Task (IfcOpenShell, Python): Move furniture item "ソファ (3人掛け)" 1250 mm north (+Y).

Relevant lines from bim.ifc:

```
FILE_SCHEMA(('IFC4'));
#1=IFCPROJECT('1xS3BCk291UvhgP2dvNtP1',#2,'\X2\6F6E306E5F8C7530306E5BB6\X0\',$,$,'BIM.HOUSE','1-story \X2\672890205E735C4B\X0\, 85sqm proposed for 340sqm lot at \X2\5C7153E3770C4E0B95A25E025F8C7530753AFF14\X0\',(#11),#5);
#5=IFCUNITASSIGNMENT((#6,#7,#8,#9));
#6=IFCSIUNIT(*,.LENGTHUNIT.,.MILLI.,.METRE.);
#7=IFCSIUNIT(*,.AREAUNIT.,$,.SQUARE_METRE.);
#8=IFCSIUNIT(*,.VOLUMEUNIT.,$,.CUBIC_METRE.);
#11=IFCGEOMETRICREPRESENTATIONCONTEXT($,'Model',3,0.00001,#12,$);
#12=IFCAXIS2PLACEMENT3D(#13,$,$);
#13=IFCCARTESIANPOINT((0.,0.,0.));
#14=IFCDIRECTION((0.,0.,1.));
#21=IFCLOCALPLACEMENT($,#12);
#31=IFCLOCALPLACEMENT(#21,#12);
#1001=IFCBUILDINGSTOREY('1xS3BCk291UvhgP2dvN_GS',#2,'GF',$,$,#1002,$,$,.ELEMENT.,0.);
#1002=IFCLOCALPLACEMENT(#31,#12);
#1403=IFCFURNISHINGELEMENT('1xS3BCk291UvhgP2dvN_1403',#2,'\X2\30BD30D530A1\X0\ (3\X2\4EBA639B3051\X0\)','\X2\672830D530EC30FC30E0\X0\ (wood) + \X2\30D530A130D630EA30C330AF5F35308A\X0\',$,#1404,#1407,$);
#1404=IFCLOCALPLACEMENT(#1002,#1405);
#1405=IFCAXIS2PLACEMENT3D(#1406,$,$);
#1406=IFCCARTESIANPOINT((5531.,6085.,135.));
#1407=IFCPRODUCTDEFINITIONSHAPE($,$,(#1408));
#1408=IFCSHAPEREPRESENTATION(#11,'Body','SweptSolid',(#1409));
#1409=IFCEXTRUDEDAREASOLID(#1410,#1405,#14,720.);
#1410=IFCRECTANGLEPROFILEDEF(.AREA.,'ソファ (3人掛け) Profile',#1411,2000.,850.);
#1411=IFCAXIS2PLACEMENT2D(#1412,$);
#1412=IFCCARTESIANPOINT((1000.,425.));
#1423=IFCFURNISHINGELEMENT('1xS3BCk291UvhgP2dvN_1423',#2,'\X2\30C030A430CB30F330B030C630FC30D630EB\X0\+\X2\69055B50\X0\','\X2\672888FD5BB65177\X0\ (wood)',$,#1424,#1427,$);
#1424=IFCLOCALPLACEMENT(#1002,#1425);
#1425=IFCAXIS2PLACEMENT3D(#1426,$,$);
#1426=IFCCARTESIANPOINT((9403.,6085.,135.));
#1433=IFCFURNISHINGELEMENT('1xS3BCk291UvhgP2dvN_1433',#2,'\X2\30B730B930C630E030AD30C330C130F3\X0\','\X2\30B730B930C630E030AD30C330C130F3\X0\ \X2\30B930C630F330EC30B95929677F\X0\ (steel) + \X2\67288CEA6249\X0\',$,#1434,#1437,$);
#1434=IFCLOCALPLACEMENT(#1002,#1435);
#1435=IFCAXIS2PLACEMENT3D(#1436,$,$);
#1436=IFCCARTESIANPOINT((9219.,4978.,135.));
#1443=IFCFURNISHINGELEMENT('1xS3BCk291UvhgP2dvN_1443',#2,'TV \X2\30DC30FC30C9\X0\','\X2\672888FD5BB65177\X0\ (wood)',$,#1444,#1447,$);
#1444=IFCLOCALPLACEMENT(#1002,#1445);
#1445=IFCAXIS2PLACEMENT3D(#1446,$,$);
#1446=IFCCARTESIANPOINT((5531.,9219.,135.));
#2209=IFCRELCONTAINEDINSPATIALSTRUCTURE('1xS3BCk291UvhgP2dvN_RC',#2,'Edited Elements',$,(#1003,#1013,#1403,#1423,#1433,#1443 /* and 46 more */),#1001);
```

```python
import ifcopenshell
import ifcopenshell.api.geometry
import ifcopenshell.util.placement
import ifcopenshell.util.unit

model = ifcopenshell.open("bim.ifc")
unit_scale = ifcopenshell.util.unit.calculate_unit_scale(model)

item = model.by_guid("1xS3BCk291UvhgP2dvN_1403")
matrix = ifcopenshell.util.placement.get_local_placement(item.ObjectPlacement)
matrix[1, 3] += 1.25 / unit_scale
ifcopenshell.api.geometry.edit_object_placement(model, product=item, matrix=matrix, is_si=False)

print(ifcopenshell.util.placement.get_local_placement(item.ObjectPlacement).round(3) + 0.0)

model.write("bim-out.ifc")
```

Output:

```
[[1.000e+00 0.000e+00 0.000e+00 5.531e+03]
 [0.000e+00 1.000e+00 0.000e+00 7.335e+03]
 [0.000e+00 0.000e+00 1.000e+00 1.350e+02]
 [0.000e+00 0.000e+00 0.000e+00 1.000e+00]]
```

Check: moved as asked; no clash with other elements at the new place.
